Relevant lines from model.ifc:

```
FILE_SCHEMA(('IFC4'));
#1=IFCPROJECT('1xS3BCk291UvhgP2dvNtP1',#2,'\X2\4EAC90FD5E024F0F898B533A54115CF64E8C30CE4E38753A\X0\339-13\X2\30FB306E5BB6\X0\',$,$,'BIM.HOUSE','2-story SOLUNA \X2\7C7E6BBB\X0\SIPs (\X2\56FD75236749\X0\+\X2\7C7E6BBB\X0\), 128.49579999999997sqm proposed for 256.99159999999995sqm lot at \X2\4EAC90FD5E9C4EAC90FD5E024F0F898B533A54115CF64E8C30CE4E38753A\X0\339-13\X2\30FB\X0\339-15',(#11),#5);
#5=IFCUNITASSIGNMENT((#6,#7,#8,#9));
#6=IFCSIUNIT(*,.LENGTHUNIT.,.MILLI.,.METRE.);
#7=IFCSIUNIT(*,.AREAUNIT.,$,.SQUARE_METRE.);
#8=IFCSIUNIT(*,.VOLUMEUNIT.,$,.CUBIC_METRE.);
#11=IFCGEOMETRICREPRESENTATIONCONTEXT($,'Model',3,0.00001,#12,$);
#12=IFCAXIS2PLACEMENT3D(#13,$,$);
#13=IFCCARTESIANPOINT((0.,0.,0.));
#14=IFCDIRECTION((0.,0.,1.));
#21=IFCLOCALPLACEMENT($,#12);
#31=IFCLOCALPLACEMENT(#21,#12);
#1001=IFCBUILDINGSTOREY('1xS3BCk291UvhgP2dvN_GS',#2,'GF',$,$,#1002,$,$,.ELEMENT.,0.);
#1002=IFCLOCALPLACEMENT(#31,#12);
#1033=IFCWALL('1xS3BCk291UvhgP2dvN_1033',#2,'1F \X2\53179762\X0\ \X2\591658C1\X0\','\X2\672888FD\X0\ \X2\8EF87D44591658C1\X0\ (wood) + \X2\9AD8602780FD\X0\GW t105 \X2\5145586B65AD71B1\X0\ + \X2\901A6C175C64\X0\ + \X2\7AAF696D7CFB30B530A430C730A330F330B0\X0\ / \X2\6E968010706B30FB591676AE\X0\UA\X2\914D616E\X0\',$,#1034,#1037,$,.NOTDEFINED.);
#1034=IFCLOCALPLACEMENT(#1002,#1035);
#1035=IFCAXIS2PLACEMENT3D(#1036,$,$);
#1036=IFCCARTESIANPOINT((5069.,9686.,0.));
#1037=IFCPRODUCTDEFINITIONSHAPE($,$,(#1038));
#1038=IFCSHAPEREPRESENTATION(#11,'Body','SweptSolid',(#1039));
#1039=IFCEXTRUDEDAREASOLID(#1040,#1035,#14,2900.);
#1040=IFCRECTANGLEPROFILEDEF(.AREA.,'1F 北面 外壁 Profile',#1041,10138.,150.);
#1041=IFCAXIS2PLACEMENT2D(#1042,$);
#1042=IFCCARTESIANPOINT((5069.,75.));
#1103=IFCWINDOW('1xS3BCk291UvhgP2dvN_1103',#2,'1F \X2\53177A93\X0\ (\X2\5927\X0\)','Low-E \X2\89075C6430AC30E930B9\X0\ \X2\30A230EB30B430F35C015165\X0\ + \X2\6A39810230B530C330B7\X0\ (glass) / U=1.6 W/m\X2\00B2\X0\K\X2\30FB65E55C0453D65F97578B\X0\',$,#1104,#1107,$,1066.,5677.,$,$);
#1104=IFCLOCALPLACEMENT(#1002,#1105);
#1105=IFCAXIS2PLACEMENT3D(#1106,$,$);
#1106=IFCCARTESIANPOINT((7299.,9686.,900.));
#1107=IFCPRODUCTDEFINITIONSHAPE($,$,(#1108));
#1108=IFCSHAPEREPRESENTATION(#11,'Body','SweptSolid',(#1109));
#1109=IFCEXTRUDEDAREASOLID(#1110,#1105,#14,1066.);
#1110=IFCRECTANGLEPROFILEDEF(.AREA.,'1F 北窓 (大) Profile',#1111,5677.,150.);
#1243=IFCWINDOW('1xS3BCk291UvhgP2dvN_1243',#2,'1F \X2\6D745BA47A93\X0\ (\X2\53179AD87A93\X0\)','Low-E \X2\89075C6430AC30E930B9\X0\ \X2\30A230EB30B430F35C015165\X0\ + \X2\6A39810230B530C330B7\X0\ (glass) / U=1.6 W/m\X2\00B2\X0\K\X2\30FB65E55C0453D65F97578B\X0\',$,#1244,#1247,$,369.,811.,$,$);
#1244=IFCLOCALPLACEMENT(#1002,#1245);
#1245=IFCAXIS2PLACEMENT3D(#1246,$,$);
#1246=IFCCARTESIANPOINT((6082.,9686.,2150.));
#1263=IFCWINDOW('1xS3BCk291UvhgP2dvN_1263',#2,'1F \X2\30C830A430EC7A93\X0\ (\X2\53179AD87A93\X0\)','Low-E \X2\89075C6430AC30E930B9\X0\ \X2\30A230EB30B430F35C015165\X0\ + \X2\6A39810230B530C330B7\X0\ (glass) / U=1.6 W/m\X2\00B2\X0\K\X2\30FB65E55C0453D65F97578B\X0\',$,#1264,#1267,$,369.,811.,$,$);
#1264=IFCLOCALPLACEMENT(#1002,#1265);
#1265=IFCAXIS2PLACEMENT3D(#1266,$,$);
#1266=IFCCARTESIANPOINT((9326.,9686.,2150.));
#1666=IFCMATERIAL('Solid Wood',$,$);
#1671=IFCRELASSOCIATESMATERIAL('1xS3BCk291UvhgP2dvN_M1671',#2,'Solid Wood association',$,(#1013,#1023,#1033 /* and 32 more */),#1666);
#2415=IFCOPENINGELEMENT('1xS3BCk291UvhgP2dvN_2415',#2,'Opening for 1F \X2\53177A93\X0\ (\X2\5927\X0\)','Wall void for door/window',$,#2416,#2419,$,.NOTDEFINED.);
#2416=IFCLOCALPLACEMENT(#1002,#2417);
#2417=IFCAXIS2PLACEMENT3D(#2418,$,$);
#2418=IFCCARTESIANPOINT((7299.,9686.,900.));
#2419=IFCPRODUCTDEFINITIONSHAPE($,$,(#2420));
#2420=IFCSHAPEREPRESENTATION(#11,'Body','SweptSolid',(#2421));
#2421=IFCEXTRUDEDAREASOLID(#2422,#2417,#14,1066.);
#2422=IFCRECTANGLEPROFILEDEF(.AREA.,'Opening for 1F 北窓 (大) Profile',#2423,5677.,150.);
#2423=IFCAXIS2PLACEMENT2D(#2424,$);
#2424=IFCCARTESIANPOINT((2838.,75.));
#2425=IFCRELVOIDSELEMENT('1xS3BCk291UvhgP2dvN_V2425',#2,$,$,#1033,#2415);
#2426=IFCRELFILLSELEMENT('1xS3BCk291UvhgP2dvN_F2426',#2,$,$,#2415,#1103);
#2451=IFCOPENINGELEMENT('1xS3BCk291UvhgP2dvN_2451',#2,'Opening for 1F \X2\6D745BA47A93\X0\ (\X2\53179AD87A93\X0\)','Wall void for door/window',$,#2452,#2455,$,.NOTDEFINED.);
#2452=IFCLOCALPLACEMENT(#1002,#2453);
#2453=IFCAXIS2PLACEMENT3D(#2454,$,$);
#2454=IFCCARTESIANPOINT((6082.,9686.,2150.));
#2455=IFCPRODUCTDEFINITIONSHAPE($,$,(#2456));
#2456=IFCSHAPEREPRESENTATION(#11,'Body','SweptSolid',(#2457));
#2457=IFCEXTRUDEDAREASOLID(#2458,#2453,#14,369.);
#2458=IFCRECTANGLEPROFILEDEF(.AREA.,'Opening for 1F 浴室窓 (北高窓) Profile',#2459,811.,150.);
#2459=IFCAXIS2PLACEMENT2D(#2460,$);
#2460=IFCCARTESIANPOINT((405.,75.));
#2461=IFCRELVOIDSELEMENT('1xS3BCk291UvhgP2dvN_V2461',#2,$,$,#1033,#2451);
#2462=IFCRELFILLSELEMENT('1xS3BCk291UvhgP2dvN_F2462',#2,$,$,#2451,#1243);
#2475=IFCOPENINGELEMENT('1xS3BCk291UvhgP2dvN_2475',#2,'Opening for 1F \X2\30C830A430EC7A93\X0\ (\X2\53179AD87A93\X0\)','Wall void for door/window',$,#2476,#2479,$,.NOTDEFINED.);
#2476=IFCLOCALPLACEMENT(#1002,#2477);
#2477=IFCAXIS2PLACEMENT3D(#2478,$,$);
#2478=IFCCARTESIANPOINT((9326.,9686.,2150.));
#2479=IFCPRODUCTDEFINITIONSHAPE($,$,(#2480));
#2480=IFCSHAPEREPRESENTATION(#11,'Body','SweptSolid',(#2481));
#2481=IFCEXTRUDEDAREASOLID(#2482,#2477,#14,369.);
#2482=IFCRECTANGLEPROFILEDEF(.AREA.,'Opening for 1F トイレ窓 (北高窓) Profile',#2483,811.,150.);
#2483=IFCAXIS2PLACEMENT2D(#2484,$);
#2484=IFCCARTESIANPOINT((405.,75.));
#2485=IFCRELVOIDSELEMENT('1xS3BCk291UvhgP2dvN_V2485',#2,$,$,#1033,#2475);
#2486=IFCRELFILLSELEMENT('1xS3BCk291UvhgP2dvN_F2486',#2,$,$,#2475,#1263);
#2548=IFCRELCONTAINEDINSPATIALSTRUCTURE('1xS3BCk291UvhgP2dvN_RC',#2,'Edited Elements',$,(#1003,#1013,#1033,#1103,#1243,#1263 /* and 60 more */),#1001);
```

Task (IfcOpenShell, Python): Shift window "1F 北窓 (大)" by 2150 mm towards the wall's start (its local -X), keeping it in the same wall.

```python
import ifcopenshell
import ifcopenshell.api.geometry
import ifcopenshell.util.placement
import ifcopenshell.util.unit

model = ifcopenshell.open("model.ifc")
unit_scale = ifcopenshell.util.unit.calculate_unit_scale(model)

window = model.by_guid("1xS3BCk291UvhgP2dvN_1103")
opening = window.FillsVoids[0].RelatingOpeningElement
wall = opening.VoidsElements[0].RelatingBuildingElement

wall_matrix = ifcopenshell.util.placement.get_local_placement(wall.ObjectPlacement)
shift = wall_matrix[:3, 0] * -2.15 / unit_scale
before = ifcopenshell.util.placement.get_local_placement(window.ObjectPlacement)[:3, 3].copy()

# The window is not placed relative to its opening, so move both.
for product in (opening, window):
    matrix = ifcopenshell.util.placement.get_local_placement(product.ObjectPlacement)
    matrix[:3, 3] += shift
    ifcopenshell.api.geometry.edit_object_placement(model, product=product, matrix=matrix, is_si=False)

after = ifcopenshell.util.placement.get_local_placement(window.ObjectPlacement)[:3, 3]
print("window moved by", (after - before).round(3) + 0.0)

model.write("model-out.ifc")
```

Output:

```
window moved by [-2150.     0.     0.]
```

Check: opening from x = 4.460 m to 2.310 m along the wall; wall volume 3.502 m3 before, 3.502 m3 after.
